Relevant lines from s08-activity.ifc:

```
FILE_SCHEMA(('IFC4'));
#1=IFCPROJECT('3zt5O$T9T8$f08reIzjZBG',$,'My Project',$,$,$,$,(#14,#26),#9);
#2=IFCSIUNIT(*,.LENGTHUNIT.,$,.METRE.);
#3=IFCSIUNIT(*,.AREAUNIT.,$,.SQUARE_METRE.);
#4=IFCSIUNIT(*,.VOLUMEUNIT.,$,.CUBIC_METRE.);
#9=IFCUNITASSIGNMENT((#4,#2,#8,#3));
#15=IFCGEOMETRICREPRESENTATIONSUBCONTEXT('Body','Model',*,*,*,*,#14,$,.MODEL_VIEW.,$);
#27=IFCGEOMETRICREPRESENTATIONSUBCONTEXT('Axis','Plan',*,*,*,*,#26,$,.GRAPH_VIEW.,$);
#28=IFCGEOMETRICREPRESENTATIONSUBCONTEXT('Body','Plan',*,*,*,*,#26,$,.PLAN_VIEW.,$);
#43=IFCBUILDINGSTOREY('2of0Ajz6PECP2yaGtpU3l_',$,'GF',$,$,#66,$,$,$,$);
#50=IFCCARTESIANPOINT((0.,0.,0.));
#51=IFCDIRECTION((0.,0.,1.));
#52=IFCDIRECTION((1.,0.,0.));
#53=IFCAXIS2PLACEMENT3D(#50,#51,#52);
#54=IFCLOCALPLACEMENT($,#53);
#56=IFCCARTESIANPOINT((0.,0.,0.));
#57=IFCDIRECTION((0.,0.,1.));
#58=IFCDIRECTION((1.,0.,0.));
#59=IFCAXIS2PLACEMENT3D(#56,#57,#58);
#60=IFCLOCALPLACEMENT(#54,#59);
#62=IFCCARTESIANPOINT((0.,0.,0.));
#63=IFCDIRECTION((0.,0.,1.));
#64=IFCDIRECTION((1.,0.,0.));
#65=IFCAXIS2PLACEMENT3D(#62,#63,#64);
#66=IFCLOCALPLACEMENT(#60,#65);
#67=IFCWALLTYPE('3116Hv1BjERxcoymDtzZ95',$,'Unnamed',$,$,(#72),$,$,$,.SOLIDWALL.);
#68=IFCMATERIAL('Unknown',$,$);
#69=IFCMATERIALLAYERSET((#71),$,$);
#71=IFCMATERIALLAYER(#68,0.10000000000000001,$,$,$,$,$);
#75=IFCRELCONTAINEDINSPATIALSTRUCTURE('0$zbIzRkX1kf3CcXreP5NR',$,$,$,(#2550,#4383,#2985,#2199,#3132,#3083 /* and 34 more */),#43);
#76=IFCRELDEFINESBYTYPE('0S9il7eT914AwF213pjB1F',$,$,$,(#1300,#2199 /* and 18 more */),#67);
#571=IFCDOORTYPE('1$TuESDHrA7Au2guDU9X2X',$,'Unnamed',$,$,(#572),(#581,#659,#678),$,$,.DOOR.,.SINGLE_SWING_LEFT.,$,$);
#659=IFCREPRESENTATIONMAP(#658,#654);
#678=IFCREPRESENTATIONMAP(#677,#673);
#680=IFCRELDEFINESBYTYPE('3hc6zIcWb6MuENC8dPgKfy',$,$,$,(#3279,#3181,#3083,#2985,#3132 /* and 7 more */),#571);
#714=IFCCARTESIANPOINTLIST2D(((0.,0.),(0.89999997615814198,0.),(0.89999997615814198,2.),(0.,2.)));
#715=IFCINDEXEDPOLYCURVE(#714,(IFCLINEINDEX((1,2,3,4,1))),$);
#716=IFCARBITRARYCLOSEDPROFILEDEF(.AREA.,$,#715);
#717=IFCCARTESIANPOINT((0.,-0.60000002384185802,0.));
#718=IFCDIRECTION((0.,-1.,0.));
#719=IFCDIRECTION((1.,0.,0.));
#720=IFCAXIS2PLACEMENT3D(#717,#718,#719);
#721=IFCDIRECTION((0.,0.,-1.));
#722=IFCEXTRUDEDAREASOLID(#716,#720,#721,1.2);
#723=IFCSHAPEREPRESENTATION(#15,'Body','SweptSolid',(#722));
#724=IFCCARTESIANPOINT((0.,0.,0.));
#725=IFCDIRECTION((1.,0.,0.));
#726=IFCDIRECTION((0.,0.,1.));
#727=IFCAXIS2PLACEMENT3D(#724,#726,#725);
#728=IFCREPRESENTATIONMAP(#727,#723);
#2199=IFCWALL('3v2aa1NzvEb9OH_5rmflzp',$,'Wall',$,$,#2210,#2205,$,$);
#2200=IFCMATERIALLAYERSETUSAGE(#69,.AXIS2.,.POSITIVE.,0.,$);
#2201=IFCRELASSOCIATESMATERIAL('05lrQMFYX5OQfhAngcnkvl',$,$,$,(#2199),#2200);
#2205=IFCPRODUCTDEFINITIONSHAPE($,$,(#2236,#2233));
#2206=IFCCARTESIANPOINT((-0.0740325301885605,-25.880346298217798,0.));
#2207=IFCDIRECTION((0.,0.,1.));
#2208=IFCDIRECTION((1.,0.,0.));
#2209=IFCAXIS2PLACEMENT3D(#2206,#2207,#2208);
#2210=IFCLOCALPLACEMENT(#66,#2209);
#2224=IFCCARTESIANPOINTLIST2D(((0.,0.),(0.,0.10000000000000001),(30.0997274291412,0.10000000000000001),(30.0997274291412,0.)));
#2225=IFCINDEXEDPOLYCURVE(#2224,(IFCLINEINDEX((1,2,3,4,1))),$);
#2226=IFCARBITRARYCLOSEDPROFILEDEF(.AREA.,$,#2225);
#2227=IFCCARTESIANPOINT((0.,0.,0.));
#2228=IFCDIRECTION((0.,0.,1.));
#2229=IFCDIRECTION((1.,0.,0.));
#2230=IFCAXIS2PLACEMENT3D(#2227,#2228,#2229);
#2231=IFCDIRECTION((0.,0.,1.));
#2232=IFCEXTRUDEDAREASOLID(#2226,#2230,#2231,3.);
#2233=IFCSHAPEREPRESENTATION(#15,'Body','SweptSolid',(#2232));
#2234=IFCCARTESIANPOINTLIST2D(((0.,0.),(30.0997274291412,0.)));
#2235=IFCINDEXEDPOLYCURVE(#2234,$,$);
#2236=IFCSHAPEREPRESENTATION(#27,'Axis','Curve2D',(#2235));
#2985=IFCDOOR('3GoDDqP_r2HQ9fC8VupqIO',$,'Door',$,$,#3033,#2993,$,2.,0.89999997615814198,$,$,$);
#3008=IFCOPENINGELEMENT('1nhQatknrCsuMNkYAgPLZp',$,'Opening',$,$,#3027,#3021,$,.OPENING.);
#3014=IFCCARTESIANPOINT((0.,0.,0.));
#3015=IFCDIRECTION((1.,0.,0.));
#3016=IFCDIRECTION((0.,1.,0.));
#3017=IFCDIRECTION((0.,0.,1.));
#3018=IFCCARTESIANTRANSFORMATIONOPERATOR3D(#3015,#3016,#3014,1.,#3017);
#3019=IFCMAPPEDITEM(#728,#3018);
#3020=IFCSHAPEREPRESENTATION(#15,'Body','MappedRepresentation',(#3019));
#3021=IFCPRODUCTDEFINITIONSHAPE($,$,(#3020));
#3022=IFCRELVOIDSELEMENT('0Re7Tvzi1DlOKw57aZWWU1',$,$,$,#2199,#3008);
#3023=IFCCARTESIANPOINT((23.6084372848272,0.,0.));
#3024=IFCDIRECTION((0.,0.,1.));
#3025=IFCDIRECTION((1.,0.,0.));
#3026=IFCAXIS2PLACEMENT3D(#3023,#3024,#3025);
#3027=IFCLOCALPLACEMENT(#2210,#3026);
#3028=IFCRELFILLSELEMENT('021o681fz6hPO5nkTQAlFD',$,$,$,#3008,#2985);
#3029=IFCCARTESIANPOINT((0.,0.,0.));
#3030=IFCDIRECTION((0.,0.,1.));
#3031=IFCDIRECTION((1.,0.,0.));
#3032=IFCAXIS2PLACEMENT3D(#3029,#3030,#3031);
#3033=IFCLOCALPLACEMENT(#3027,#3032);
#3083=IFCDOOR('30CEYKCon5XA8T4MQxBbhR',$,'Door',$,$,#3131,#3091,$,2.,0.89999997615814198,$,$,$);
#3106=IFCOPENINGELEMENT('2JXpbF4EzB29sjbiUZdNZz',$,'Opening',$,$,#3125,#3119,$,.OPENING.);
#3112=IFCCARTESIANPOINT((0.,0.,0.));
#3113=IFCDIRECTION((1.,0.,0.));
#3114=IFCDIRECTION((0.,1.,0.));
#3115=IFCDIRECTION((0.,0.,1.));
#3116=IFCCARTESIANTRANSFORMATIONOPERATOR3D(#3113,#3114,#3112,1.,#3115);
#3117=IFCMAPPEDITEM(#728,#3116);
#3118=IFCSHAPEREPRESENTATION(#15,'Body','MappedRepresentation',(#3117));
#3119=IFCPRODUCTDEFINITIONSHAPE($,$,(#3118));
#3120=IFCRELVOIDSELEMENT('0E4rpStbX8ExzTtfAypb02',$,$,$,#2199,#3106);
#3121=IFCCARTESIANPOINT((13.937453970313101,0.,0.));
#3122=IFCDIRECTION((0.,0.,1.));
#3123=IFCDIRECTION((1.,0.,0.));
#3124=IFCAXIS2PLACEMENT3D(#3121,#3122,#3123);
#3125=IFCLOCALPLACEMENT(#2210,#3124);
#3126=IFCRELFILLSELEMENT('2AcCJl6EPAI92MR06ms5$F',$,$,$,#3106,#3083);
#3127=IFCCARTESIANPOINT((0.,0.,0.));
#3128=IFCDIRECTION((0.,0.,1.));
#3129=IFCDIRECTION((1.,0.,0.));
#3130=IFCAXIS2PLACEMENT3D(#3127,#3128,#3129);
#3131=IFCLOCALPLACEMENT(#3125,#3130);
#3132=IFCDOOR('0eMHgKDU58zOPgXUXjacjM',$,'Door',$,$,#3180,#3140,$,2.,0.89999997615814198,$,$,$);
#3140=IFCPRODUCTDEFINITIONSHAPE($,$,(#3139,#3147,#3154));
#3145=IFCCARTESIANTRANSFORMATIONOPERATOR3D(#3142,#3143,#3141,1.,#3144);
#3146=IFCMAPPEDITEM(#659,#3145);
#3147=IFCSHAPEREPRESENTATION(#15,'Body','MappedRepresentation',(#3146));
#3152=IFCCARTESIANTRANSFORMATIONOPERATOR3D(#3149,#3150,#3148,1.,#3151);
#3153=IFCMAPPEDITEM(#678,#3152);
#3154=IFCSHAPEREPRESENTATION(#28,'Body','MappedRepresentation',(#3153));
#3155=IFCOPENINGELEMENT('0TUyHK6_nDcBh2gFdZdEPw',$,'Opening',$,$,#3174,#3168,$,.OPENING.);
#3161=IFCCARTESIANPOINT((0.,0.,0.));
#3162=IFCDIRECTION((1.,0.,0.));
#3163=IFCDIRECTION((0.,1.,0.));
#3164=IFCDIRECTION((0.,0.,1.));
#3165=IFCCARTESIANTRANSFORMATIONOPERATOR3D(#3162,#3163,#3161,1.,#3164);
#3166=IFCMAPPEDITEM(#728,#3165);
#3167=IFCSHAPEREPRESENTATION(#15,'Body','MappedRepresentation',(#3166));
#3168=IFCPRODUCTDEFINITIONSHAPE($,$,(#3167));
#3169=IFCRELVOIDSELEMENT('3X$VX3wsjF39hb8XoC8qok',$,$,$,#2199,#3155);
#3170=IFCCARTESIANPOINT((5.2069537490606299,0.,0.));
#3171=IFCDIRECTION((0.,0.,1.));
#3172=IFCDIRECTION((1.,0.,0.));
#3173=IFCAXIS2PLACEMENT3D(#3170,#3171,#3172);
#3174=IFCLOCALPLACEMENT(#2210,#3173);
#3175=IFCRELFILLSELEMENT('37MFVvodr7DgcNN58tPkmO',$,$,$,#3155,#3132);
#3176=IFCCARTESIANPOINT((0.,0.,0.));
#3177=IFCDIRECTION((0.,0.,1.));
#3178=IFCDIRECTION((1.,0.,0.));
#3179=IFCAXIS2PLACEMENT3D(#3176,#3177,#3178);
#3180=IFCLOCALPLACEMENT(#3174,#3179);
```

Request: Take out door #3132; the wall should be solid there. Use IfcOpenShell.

```python
import ifcopenshell
import ifcopenshell.api.feature
import ifcopenshell.api.root
import ifcopenshell.geom
import ifcopenshell.util.shape

model = ifcopenshell.open("s08-activity.ifc")
settings = ifcopenshell.geom.settings()


def volume(element):
    """Net volume in cubic metres, openings subtracted."""
    shape = ifcopenshell.geom.create_shape(settings, element)
    return ifcopenshell.util.shape.get_volume(shape.geometry)


door = model.by_guid("0eMHgKDU58zOPgXUXjacjM")
opening = door.FillsVoids[0].RelatingOpeningElement
wall = opening.VoidsElements[0].RelatingBuildingElement
before = volume(wall)

ifcopenshell.api.root.remove_product(model, product=door)
ifcopenshell.api.feature.remove_feature(model, feature=opening)

after = volume(wall)

print(f"wall volume {before:.3f} -> {after:.3f} m3")

model.write("s08-activity_updated.ifc")
```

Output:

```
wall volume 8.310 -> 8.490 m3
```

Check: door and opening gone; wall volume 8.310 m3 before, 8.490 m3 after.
